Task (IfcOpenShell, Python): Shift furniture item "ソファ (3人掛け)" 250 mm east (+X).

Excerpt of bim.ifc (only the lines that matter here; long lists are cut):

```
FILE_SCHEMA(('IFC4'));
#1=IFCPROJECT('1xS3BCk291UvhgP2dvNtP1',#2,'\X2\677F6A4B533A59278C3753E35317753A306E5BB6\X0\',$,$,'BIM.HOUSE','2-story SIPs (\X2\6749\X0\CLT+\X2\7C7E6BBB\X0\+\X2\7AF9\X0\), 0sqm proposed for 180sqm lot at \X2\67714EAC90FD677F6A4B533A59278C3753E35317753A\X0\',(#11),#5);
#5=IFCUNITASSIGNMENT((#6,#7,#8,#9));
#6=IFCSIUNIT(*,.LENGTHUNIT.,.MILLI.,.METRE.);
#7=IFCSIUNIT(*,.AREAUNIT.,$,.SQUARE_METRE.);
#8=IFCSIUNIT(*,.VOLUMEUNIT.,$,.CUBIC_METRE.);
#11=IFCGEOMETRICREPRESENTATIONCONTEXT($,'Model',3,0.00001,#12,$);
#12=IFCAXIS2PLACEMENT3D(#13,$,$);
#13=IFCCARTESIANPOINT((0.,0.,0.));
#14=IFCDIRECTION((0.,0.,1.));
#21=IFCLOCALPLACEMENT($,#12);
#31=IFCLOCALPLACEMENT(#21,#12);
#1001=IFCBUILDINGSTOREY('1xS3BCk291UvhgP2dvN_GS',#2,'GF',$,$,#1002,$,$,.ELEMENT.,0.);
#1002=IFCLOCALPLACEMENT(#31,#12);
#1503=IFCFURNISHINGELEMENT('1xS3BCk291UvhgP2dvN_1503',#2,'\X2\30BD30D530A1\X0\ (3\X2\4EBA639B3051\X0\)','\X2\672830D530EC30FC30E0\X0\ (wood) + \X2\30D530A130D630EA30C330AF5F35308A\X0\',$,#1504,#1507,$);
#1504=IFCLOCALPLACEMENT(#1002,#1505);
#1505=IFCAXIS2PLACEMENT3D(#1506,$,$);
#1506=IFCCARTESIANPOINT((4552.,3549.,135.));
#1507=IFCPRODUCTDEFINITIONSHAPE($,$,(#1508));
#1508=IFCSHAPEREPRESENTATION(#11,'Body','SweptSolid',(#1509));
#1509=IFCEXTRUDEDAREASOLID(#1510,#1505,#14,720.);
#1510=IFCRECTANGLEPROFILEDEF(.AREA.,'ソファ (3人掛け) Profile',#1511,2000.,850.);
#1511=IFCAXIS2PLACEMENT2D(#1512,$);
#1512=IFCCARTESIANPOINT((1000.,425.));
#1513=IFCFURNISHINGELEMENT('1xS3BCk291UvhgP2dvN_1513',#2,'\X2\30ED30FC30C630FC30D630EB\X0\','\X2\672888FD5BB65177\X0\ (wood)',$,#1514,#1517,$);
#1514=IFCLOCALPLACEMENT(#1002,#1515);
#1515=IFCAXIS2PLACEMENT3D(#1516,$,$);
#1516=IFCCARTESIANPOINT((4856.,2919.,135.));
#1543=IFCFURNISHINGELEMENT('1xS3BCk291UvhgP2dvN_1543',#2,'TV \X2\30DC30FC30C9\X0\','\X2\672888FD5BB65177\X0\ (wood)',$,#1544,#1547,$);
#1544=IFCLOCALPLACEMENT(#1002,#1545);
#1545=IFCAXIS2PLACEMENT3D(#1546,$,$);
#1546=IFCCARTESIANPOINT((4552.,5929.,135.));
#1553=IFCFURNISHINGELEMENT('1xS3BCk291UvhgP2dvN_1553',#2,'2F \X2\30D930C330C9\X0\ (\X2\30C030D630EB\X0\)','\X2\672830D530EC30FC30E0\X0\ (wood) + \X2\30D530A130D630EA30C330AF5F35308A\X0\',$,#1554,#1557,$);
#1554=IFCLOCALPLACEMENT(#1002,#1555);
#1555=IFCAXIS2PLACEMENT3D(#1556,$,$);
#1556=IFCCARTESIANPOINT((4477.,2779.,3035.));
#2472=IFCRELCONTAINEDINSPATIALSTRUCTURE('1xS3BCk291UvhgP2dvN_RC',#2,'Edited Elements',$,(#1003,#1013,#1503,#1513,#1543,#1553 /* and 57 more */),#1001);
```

```python
import ifcopenshell
import ifcopenshell.api.geometry
import ifcopenshell.util.placement
import ifcopenshell.util.unit

model = ifcopenshell.open("bim.ifc")
unit_scale = ifcopenshell.util.unit.calculate_unit_scale(model)

item = model.by_guid("1xS3BCk291UvhgP2dvN_1503")
matrix = ifcopenshell.util.placement.get_local_placement(item.ObjectPlacement)
matrix[0, 3] += 0.25 / unit_scale
ifcopenshell.api.geometry.edit_object_placement(model, product=item, matrix=matrix, is_si=False)

print(ifcopenshell.util.placement.get_local_placement(item.ObjectPlacement).round(3) + 0.0)

model.write("bim_rev.ifc")
```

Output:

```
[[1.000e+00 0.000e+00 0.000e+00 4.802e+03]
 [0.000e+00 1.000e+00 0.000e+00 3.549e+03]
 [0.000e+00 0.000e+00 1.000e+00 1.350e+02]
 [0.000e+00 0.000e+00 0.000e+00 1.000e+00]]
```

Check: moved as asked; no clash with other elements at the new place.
